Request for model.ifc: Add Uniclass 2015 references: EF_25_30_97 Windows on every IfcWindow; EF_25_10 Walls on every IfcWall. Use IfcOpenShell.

First a look at what the model holds.

```python
import ifcopenshell

model = ifcopenshell.open("model.ifc")
print(model.schema)
print("classifications:", [c.Name for c in model.by_type("IfcClassification")])
for ifc_class in ("IfcDoor", "IfcRoof", "IfcStair", "IfcWall", "IfcWindow"):
    print(ifc_class, len(model.by_type(ifc_class)))
```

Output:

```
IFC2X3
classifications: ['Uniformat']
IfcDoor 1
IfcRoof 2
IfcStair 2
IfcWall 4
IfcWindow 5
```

```python
import ifcopenshell
import ifcopenshell.api.classification

model = ifcopenshell.open("model.ifc")

# IFC2X3 requires Source and Edition and has no link from the project to the system.
system = model.create_entity("IfcClassification", Source="NBS", Edition="2015", Name="Uniclass 2015")

codes = {
    "IfcWindow": ("EF_25_30_97", "Windows"),
    "IfcWall": ("EF_25_10", "Walls"),
}
for ifc_class, (code, name) in codes.items():
    products = model.by_type(ifc_class)
    ifcopenshell.api.classification.add_reference(
        model, products=products, classification=system, identification=code, name=name
    )
    print(code, len(products))

model.write("model_edited.ifc")
```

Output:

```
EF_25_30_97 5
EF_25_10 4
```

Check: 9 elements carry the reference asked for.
